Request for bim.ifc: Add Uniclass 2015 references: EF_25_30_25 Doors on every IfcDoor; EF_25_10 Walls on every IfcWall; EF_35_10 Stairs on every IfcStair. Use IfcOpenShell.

First a look at what the model holds.

```python
import ifcopenshell

model = ifcopenshell.open("bim.ifc")
print(model.schema)
print("classifications:", [c.Name for c in model.by_type("IfcClassification")])
for ifc_class in ("IfcDoor", "IfcRoof", "IfcStair", "IfcWall", "IfcWindow"):
    print(ifc_class, len(model.by_type(ifc_class)))
```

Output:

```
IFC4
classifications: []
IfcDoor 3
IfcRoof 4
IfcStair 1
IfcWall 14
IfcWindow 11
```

```python
import ifcopenshell
import ifcopenshell.api.classification

model = ifcopenshell.open("bim.ifc")

system = ifcopenshell.api.classification.add_classification(model, classification="Uniclass 2015")

codes = {
    "IfcDoor": ("EF_25_30_25", "Doors"),
    "IfcWall": ("EF_25_10", "Walls"),
    "IfcStair": ("EF_35_10", "Stairs"),
}
for ifc_class, (code, name) in codes.items():
    products = model.by_type(ifc_class)
    ifcopenshell.api.classification.add_reference(
        model, products=products, classification=system, identification=code, name=name
    )
    print(code, len(products))

model.write("bim_edited.ifc")
```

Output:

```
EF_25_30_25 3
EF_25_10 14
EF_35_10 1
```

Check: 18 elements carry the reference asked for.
